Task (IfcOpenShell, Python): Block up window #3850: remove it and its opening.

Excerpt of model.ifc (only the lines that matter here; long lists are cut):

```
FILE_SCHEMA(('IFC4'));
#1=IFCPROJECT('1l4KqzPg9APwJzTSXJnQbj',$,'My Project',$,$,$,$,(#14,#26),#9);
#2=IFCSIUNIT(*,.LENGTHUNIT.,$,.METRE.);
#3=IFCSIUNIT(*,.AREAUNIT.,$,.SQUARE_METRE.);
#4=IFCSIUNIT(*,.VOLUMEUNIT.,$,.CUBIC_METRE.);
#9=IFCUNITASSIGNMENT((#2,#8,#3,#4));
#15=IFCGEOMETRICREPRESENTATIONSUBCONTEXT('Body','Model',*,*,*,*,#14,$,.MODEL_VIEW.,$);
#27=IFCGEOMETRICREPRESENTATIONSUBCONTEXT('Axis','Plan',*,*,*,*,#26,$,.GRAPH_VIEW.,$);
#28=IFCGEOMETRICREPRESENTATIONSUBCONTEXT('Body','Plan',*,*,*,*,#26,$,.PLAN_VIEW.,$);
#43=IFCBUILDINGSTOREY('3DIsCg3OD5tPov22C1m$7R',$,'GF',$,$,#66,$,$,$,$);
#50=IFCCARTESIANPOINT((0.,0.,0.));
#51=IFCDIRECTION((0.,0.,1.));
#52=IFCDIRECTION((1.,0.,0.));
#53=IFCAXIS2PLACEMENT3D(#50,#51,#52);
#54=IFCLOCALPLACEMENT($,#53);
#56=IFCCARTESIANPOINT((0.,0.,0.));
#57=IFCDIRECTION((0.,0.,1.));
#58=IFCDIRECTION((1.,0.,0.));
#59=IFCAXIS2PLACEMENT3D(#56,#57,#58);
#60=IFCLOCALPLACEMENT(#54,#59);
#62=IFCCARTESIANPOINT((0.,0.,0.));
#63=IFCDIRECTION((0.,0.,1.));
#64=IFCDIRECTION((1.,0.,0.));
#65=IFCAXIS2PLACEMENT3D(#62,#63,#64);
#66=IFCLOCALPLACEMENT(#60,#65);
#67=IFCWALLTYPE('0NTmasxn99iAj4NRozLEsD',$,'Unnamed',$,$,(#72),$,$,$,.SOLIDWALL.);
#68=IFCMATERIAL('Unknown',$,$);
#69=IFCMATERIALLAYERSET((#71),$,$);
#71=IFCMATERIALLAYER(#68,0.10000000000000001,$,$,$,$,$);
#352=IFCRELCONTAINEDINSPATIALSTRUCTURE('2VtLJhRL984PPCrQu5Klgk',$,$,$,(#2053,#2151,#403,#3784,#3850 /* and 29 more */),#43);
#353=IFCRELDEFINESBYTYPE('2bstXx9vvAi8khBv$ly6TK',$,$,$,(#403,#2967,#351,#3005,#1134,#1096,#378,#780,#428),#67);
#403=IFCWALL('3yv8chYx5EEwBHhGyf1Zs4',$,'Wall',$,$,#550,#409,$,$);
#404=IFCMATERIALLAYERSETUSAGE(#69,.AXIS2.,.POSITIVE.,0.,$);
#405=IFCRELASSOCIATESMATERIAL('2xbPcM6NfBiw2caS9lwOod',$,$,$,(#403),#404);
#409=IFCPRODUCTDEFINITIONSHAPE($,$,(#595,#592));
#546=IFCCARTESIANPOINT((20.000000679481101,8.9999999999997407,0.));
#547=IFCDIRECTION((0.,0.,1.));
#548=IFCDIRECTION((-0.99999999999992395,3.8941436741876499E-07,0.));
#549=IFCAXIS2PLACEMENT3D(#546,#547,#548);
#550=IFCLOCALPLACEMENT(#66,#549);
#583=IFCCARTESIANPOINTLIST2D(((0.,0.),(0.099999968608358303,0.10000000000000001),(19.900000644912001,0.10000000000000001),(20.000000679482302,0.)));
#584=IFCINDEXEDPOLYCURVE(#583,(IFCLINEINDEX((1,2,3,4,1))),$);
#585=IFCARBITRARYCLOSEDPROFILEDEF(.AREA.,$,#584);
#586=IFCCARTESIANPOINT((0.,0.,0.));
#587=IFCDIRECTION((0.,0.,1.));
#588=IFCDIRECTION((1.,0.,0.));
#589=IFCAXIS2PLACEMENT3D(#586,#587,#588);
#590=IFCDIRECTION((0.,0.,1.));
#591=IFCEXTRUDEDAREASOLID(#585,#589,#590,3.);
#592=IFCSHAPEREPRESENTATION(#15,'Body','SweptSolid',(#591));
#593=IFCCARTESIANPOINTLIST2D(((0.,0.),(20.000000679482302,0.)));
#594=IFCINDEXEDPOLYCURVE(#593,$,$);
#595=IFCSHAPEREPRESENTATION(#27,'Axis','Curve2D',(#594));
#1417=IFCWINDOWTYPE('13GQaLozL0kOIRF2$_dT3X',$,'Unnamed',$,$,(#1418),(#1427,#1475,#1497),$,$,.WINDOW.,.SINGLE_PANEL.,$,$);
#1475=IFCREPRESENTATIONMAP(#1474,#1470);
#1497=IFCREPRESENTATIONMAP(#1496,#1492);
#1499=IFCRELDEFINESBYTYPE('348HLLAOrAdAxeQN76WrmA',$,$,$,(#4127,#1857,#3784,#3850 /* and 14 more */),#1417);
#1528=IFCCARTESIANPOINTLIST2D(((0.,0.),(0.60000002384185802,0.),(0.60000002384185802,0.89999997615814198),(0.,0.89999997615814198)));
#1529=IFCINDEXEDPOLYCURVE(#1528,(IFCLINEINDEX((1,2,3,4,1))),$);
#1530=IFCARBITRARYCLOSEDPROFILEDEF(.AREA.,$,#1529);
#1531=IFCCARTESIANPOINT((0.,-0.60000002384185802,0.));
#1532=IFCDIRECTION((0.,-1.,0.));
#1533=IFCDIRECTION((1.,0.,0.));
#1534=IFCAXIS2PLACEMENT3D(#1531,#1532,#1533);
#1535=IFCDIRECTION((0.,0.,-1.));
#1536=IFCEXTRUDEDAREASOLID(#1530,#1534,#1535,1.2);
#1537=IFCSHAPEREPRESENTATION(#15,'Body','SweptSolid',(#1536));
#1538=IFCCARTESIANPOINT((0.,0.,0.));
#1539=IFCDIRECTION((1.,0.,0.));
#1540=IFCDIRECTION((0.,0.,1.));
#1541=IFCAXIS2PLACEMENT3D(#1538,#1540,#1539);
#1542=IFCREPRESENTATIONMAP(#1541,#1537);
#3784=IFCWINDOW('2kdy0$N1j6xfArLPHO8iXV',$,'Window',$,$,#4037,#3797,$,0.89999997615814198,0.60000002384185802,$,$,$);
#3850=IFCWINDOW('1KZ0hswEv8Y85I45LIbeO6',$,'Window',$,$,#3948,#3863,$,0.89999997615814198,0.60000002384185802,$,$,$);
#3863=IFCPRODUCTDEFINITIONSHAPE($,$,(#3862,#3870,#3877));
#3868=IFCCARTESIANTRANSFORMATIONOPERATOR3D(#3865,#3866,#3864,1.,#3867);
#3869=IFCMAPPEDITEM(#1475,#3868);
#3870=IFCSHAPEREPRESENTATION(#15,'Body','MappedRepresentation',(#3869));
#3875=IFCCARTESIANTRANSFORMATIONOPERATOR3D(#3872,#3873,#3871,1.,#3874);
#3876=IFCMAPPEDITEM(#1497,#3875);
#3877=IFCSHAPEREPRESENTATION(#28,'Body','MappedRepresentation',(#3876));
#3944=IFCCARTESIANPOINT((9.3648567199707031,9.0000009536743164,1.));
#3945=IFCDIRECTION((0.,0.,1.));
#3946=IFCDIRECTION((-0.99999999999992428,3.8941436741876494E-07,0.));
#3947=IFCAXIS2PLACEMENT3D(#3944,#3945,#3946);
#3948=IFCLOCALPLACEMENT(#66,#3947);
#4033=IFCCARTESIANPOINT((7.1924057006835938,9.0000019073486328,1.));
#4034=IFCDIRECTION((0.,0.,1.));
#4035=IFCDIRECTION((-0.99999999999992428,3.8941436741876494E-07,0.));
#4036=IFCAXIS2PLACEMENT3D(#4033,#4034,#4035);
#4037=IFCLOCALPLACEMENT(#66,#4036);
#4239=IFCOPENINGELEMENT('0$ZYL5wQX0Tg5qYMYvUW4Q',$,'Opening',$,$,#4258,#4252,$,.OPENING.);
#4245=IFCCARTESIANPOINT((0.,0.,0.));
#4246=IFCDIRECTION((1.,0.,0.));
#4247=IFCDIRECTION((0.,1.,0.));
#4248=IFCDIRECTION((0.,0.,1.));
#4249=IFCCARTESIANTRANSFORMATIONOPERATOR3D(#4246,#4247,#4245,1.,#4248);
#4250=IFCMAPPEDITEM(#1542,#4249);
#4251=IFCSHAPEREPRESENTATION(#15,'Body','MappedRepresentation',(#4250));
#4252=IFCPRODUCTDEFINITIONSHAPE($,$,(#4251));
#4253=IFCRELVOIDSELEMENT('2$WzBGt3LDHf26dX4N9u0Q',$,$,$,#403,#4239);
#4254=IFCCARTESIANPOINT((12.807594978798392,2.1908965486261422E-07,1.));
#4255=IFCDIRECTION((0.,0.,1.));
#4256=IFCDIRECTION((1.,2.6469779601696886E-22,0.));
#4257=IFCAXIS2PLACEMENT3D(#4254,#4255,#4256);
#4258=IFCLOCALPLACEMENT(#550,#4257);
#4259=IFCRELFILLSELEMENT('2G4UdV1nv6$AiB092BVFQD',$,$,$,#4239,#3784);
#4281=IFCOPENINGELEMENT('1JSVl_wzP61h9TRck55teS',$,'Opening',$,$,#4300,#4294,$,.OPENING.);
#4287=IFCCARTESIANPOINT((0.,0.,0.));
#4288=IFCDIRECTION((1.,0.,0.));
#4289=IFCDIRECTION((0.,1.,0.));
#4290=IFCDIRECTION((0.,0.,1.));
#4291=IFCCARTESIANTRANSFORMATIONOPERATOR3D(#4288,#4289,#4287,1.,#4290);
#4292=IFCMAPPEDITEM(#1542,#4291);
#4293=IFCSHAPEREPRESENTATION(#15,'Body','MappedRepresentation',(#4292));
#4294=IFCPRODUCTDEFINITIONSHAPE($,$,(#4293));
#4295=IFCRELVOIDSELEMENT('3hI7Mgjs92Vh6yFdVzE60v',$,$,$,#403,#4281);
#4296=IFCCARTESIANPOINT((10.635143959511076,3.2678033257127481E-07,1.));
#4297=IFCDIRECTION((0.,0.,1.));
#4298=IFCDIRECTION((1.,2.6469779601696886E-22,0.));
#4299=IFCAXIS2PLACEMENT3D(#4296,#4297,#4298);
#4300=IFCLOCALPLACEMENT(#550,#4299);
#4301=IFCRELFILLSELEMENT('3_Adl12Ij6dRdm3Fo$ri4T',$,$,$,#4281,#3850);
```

```python
import ifcopenshell
import ifcopenshell.api.feature
import ifcopenshell.api.root
import ifcopenshell.geom
import ifcopenshell.util.shape

model = ifcopenshell.open("model.ifc")
settings = ifcopenshell.geom.settings()


def volume(element):
    """Net volume in cubic metres, openings subtracted."""
    shape = ifcopenshell.geom.create_shape(settings, element)
    return ifcopenshell.util.shape.get_volume(shape.geometry)


window = model.by_guid("1KZ0hswEv8Y85I45LIbeO6")
opening = window.FillsVoids[0].RelatingOpeningElement
wall = opening.VoidsElements[0].RelatingBuildingElement
before = volume(wall)

ifcopenshell.api.root.remove_product(model, product=window)
ifcopenshell.api.feature.remove_feature(model, feature=opening)

after = volume(wall)

print(f"wall volume {before:.3f} -> {after:.3f} m3")

model.write("model_updated.ifc")
```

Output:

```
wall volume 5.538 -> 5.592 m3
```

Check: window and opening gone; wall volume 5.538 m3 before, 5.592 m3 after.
